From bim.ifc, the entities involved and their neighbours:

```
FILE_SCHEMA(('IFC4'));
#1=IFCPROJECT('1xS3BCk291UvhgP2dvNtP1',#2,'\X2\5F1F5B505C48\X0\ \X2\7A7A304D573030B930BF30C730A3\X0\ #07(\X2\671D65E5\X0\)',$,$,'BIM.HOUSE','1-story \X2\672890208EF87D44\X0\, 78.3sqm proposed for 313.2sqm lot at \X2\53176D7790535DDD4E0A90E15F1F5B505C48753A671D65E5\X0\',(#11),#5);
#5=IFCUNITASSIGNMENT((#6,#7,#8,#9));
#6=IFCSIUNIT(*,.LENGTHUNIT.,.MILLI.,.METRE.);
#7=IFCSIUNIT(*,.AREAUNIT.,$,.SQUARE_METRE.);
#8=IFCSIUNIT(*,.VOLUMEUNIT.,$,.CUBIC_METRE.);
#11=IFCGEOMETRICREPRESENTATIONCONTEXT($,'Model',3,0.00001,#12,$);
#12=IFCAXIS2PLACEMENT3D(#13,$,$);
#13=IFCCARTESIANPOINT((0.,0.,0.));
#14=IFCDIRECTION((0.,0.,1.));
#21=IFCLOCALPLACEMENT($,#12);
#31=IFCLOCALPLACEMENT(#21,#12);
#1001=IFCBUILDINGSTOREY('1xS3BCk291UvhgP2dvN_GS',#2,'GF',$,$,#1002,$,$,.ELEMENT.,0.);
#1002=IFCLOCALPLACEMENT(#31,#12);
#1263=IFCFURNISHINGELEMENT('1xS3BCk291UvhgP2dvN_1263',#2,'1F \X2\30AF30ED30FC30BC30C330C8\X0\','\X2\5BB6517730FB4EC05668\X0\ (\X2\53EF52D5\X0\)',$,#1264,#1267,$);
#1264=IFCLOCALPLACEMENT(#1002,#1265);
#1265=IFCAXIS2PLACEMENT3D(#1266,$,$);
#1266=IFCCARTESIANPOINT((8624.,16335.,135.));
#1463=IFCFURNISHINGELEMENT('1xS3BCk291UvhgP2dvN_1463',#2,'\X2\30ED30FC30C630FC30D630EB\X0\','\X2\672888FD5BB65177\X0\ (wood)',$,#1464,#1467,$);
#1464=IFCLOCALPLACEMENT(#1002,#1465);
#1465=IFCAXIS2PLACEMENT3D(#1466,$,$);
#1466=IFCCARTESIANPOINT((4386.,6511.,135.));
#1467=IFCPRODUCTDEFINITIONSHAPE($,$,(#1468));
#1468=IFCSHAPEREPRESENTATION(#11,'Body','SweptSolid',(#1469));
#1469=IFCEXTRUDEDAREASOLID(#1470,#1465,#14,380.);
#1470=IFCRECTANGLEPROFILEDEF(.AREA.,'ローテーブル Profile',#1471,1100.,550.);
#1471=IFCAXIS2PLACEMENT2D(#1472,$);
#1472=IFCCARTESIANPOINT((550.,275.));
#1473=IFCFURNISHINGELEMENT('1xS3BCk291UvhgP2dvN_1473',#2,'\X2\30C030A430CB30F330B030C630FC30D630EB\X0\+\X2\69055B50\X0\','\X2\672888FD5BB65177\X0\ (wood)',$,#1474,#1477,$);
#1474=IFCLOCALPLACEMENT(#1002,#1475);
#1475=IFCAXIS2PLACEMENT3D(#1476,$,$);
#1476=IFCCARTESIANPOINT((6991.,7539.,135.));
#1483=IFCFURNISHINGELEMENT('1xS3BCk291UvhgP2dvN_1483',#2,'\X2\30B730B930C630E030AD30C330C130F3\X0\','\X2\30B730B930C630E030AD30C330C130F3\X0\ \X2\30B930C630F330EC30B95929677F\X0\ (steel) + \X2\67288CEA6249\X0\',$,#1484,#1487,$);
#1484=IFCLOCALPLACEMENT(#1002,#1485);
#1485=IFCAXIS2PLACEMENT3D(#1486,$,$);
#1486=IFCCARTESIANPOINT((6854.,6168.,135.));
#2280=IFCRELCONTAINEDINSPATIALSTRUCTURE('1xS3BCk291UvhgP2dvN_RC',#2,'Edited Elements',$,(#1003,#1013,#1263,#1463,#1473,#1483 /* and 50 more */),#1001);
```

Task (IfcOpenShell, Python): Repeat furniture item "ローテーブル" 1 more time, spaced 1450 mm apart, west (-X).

```python
import numpy as np
import ifcopenshell
import ifcopenshell.api.geometry
import ifcopenshell.api.root
import ifcopenshell.util.element
import ifcopenshell.util.placement
import ifcopenshell.util.unit

model = ifcopenshell.open("bim.ifc")
unit_scale = ifcopenshell.util.unit.calculate_unit_scale(model)


def reuse_history(source, copy):
    """copy_class also copies each property set's owner history, people and application; keep the originals."""
    for rel in copy.IsDefinedBy:
        if rel.is_a("IfcRelDefinesByProperties") and (history := rel.RelatingPropertyDefinition.OwnerHistory):
            rel.RelatingPropertyDefinition.OwnerHistory = source.OwnerHistory
            ifcopenshell.util.element.remove_deep2(model, history)


source = model.by_guid("1xS3BCk291UvhgP2dvN_1463")
base = ifcopenshell.util.placement.get_local_placement(source.ObjectPlacement)
step = np.array([-1.0, 0.0, 0.0]) * 1.45 / unit_scale

for i in range(1, 2):
    copy = ifcopenshell.api.root.copy_class(model, product=source)
    copy.Representation = ifcopenshell.util.element.copy_deep(
        model, source.Representation, exclude=["IfcGeometricRepresentationContext", "IfcRepresentationMap"]
    )
    reuse_history(source, copy)
    matrix = base.copy()
    matrix[:3, 3] += i * step
    print("added at", matrix[:3, 3].round(3) + 0.0)
    ifcopenshell.api.geometry.edit_object_placement(model, product=copy, matrix=matrix, is_si=False)

model.write("bim_rev.ifc")
```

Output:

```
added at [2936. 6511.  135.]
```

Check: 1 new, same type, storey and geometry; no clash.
